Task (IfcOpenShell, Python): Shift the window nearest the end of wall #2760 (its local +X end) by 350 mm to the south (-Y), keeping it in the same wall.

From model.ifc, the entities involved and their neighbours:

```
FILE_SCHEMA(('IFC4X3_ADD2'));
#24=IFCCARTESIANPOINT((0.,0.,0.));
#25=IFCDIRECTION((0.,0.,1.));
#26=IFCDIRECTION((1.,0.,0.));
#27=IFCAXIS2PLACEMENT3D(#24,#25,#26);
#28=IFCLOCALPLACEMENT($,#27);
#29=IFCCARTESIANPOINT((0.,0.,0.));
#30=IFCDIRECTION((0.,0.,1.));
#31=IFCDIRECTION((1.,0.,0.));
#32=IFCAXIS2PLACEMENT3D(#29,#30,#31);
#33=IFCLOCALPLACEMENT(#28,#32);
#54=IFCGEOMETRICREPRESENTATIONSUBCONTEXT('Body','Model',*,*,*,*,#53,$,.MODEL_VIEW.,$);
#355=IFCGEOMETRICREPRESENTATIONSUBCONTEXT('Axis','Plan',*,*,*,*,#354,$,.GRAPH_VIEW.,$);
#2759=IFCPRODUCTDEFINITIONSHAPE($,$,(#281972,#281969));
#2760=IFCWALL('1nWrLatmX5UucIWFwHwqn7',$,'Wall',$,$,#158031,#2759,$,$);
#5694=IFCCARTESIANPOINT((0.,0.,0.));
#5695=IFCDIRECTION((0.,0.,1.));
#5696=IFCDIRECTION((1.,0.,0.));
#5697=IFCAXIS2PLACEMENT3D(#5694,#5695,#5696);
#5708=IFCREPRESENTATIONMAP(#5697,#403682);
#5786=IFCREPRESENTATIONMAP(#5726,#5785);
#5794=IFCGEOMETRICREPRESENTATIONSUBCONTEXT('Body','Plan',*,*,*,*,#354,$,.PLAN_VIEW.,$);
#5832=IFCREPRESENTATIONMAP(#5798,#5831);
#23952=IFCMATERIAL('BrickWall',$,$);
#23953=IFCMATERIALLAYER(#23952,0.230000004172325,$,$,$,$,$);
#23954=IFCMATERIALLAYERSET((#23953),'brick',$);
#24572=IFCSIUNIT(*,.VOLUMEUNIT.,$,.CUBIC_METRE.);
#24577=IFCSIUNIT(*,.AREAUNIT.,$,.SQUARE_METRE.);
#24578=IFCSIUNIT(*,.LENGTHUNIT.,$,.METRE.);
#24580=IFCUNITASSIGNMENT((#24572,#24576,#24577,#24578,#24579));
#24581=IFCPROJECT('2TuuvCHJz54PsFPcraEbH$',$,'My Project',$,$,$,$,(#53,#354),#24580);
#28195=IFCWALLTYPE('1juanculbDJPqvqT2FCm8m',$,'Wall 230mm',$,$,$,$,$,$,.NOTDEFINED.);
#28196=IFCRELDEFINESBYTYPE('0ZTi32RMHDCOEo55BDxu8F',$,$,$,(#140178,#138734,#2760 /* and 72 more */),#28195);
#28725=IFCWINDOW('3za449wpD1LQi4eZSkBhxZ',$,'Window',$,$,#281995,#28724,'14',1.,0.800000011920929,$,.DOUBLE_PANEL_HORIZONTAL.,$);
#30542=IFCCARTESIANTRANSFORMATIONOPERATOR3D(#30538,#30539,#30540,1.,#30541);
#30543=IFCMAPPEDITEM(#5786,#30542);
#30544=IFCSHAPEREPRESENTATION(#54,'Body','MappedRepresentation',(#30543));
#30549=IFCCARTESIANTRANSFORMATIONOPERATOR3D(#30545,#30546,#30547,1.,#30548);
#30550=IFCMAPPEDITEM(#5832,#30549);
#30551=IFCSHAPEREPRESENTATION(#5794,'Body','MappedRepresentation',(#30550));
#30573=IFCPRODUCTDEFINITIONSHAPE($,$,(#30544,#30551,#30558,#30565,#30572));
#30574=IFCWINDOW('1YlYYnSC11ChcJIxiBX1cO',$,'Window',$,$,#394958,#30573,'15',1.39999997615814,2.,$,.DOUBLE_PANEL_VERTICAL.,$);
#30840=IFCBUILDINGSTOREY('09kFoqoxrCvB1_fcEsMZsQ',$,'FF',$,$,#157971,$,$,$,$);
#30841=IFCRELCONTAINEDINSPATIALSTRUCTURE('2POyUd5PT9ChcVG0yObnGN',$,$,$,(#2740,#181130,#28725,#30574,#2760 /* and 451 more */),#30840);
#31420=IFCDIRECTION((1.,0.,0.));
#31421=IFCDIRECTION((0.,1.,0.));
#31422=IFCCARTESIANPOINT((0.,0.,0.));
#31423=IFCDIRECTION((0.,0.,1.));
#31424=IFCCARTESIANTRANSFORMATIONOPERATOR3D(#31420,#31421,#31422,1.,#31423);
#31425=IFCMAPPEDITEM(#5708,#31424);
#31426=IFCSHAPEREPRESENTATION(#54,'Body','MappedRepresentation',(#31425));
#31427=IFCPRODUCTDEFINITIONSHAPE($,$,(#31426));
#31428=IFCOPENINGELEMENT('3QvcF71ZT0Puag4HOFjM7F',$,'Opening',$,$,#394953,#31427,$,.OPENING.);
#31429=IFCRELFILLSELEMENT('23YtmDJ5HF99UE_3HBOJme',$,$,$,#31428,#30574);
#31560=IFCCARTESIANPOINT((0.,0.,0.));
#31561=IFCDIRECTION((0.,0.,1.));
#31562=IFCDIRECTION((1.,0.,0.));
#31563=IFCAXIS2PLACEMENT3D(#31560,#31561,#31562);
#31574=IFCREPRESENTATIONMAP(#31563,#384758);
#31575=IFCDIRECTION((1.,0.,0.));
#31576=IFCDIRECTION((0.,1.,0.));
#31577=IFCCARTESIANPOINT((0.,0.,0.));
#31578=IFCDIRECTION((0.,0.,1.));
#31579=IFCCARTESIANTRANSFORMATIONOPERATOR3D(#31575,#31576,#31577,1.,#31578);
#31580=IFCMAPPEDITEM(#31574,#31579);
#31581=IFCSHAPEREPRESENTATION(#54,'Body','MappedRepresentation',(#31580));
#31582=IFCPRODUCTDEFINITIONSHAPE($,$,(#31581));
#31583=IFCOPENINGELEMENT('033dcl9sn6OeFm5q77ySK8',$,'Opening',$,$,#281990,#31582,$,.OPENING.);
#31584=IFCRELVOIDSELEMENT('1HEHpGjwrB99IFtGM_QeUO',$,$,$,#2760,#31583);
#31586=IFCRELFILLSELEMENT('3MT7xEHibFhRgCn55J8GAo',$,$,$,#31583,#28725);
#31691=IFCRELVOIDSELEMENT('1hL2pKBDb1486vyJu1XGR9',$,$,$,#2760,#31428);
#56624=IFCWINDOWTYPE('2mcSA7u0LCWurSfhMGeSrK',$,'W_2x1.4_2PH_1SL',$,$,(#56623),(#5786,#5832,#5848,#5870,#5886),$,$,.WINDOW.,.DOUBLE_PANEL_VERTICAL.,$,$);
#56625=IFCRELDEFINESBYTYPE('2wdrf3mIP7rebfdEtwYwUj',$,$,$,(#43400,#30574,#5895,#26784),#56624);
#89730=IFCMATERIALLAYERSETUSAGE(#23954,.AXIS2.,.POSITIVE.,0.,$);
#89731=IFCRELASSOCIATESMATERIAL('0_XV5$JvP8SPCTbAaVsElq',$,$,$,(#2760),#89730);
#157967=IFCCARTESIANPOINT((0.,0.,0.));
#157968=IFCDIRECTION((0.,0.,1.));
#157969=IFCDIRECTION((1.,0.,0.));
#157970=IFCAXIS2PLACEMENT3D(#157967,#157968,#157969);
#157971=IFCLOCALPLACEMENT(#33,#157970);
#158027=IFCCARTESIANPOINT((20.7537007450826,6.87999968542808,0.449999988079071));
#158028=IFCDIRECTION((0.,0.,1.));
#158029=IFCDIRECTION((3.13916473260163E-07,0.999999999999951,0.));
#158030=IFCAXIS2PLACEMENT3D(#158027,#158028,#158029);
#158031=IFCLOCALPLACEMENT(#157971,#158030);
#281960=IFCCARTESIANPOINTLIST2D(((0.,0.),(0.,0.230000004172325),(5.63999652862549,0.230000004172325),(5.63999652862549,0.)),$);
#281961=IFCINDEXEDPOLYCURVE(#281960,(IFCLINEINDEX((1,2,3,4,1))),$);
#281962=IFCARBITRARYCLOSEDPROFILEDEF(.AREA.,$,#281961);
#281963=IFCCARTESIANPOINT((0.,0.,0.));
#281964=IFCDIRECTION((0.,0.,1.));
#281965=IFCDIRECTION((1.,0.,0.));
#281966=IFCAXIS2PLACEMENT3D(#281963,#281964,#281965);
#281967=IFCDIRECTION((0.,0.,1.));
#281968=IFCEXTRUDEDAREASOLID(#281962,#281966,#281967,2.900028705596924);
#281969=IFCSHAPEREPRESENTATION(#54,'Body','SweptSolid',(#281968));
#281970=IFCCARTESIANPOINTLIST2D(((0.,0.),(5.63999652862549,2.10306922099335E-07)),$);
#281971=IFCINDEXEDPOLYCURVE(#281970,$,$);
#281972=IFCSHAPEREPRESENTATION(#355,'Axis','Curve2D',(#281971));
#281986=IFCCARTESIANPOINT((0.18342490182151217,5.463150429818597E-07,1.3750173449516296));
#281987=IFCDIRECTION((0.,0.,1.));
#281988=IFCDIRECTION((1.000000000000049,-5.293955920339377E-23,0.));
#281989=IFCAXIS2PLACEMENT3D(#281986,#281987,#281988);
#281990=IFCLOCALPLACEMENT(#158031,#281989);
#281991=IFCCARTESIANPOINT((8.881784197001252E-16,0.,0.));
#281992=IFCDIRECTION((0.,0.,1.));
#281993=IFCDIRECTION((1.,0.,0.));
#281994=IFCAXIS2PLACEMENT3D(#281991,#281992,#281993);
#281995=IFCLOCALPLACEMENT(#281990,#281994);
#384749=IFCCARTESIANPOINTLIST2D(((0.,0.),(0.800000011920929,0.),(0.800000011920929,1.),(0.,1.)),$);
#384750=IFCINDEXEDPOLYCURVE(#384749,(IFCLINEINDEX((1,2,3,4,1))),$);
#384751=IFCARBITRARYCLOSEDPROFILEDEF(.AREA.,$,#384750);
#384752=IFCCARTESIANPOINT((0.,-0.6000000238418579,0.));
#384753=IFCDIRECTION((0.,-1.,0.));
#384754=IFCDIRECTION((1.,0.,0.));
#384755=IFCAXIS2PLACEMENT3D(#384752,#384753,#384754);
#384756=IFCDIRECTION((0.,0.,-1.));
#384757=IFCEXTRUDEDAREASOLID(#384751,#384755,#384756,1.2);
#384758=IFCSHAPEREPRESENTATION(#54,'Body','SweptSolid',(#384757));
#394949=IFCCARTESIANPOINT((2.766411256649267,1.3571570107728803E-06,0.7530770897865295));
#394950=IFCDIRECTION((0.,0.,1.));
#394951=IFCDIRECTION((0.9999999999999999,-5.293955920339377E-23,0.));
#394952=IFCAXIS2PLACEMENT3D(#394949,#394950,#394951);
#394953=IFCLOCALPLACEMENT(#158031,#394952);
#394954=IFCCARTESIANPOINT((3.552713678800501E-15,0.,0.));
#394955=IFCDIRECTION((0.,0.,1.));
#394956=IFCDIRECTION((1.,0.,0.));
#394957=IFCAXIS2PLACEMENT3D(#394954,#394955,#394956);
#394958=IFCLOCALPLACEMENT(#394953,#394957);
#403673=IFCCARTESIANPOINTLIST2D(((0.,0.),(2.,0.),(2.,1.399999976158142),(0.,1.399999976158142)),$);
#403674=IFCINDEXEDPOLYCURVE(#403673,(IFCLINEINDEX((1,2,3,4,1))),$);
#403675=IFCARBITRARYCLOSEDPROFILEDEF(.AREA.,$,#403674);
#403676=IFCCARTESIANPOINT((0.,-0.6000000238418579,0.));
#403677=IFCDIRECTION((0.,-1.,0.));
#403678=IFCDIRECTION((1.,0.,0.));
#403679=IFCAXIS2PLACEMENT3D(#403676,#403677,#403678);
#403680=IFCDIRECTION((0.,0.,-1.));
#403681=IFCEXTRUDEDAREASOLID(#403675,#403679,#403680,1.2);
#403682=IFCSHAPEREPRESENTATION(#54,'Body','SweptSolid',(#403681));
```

```python
import ifcopenshell
import ifcopenshell.api.geometry
import ifcopenshell.util.placement

model = ifcopenshell.open("model.ifc")

window = model.by_guid("1YlYYnSC11ChcJIxiBX1cO")
opening = window.FillsVoids[0].RelatingOpeningElement
wall = opening.VoidsElements[0].RelatingBuildingElement

wall_matrix = ifcopenshell.util.placement.get_local_placement(wall.ObjectPlacement)
shift = wall_matrix[:3, 0] * -0.35
before = ifcopenshell.util.placement.get_local_placement(window.ObjectPlacement)[:3, 3].copy()

# The window is placed relative to its opening, so it follows when the opening moves.
matrix = ifcopenshell.util.placement.get_local_placement(opening.ObjectPlacement)
matrix[:3, 3] += shift
ifcopenshell.api.geometry.edit_object_placement(
    model, product=opening, matrix=matrix, is_si=False, should_transform_children=True
)

after = ifcopenshell.util.placement.get_local_placement(window.ObjectPlacement)[:3, 3]
print("window moved by", (after - before).round(3) + 0.0)

model.write("model_edited.ifc")
```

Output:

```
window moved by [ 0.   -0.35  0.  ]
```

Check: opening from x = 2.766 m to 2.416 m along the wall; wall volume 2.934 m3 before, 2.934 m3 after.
